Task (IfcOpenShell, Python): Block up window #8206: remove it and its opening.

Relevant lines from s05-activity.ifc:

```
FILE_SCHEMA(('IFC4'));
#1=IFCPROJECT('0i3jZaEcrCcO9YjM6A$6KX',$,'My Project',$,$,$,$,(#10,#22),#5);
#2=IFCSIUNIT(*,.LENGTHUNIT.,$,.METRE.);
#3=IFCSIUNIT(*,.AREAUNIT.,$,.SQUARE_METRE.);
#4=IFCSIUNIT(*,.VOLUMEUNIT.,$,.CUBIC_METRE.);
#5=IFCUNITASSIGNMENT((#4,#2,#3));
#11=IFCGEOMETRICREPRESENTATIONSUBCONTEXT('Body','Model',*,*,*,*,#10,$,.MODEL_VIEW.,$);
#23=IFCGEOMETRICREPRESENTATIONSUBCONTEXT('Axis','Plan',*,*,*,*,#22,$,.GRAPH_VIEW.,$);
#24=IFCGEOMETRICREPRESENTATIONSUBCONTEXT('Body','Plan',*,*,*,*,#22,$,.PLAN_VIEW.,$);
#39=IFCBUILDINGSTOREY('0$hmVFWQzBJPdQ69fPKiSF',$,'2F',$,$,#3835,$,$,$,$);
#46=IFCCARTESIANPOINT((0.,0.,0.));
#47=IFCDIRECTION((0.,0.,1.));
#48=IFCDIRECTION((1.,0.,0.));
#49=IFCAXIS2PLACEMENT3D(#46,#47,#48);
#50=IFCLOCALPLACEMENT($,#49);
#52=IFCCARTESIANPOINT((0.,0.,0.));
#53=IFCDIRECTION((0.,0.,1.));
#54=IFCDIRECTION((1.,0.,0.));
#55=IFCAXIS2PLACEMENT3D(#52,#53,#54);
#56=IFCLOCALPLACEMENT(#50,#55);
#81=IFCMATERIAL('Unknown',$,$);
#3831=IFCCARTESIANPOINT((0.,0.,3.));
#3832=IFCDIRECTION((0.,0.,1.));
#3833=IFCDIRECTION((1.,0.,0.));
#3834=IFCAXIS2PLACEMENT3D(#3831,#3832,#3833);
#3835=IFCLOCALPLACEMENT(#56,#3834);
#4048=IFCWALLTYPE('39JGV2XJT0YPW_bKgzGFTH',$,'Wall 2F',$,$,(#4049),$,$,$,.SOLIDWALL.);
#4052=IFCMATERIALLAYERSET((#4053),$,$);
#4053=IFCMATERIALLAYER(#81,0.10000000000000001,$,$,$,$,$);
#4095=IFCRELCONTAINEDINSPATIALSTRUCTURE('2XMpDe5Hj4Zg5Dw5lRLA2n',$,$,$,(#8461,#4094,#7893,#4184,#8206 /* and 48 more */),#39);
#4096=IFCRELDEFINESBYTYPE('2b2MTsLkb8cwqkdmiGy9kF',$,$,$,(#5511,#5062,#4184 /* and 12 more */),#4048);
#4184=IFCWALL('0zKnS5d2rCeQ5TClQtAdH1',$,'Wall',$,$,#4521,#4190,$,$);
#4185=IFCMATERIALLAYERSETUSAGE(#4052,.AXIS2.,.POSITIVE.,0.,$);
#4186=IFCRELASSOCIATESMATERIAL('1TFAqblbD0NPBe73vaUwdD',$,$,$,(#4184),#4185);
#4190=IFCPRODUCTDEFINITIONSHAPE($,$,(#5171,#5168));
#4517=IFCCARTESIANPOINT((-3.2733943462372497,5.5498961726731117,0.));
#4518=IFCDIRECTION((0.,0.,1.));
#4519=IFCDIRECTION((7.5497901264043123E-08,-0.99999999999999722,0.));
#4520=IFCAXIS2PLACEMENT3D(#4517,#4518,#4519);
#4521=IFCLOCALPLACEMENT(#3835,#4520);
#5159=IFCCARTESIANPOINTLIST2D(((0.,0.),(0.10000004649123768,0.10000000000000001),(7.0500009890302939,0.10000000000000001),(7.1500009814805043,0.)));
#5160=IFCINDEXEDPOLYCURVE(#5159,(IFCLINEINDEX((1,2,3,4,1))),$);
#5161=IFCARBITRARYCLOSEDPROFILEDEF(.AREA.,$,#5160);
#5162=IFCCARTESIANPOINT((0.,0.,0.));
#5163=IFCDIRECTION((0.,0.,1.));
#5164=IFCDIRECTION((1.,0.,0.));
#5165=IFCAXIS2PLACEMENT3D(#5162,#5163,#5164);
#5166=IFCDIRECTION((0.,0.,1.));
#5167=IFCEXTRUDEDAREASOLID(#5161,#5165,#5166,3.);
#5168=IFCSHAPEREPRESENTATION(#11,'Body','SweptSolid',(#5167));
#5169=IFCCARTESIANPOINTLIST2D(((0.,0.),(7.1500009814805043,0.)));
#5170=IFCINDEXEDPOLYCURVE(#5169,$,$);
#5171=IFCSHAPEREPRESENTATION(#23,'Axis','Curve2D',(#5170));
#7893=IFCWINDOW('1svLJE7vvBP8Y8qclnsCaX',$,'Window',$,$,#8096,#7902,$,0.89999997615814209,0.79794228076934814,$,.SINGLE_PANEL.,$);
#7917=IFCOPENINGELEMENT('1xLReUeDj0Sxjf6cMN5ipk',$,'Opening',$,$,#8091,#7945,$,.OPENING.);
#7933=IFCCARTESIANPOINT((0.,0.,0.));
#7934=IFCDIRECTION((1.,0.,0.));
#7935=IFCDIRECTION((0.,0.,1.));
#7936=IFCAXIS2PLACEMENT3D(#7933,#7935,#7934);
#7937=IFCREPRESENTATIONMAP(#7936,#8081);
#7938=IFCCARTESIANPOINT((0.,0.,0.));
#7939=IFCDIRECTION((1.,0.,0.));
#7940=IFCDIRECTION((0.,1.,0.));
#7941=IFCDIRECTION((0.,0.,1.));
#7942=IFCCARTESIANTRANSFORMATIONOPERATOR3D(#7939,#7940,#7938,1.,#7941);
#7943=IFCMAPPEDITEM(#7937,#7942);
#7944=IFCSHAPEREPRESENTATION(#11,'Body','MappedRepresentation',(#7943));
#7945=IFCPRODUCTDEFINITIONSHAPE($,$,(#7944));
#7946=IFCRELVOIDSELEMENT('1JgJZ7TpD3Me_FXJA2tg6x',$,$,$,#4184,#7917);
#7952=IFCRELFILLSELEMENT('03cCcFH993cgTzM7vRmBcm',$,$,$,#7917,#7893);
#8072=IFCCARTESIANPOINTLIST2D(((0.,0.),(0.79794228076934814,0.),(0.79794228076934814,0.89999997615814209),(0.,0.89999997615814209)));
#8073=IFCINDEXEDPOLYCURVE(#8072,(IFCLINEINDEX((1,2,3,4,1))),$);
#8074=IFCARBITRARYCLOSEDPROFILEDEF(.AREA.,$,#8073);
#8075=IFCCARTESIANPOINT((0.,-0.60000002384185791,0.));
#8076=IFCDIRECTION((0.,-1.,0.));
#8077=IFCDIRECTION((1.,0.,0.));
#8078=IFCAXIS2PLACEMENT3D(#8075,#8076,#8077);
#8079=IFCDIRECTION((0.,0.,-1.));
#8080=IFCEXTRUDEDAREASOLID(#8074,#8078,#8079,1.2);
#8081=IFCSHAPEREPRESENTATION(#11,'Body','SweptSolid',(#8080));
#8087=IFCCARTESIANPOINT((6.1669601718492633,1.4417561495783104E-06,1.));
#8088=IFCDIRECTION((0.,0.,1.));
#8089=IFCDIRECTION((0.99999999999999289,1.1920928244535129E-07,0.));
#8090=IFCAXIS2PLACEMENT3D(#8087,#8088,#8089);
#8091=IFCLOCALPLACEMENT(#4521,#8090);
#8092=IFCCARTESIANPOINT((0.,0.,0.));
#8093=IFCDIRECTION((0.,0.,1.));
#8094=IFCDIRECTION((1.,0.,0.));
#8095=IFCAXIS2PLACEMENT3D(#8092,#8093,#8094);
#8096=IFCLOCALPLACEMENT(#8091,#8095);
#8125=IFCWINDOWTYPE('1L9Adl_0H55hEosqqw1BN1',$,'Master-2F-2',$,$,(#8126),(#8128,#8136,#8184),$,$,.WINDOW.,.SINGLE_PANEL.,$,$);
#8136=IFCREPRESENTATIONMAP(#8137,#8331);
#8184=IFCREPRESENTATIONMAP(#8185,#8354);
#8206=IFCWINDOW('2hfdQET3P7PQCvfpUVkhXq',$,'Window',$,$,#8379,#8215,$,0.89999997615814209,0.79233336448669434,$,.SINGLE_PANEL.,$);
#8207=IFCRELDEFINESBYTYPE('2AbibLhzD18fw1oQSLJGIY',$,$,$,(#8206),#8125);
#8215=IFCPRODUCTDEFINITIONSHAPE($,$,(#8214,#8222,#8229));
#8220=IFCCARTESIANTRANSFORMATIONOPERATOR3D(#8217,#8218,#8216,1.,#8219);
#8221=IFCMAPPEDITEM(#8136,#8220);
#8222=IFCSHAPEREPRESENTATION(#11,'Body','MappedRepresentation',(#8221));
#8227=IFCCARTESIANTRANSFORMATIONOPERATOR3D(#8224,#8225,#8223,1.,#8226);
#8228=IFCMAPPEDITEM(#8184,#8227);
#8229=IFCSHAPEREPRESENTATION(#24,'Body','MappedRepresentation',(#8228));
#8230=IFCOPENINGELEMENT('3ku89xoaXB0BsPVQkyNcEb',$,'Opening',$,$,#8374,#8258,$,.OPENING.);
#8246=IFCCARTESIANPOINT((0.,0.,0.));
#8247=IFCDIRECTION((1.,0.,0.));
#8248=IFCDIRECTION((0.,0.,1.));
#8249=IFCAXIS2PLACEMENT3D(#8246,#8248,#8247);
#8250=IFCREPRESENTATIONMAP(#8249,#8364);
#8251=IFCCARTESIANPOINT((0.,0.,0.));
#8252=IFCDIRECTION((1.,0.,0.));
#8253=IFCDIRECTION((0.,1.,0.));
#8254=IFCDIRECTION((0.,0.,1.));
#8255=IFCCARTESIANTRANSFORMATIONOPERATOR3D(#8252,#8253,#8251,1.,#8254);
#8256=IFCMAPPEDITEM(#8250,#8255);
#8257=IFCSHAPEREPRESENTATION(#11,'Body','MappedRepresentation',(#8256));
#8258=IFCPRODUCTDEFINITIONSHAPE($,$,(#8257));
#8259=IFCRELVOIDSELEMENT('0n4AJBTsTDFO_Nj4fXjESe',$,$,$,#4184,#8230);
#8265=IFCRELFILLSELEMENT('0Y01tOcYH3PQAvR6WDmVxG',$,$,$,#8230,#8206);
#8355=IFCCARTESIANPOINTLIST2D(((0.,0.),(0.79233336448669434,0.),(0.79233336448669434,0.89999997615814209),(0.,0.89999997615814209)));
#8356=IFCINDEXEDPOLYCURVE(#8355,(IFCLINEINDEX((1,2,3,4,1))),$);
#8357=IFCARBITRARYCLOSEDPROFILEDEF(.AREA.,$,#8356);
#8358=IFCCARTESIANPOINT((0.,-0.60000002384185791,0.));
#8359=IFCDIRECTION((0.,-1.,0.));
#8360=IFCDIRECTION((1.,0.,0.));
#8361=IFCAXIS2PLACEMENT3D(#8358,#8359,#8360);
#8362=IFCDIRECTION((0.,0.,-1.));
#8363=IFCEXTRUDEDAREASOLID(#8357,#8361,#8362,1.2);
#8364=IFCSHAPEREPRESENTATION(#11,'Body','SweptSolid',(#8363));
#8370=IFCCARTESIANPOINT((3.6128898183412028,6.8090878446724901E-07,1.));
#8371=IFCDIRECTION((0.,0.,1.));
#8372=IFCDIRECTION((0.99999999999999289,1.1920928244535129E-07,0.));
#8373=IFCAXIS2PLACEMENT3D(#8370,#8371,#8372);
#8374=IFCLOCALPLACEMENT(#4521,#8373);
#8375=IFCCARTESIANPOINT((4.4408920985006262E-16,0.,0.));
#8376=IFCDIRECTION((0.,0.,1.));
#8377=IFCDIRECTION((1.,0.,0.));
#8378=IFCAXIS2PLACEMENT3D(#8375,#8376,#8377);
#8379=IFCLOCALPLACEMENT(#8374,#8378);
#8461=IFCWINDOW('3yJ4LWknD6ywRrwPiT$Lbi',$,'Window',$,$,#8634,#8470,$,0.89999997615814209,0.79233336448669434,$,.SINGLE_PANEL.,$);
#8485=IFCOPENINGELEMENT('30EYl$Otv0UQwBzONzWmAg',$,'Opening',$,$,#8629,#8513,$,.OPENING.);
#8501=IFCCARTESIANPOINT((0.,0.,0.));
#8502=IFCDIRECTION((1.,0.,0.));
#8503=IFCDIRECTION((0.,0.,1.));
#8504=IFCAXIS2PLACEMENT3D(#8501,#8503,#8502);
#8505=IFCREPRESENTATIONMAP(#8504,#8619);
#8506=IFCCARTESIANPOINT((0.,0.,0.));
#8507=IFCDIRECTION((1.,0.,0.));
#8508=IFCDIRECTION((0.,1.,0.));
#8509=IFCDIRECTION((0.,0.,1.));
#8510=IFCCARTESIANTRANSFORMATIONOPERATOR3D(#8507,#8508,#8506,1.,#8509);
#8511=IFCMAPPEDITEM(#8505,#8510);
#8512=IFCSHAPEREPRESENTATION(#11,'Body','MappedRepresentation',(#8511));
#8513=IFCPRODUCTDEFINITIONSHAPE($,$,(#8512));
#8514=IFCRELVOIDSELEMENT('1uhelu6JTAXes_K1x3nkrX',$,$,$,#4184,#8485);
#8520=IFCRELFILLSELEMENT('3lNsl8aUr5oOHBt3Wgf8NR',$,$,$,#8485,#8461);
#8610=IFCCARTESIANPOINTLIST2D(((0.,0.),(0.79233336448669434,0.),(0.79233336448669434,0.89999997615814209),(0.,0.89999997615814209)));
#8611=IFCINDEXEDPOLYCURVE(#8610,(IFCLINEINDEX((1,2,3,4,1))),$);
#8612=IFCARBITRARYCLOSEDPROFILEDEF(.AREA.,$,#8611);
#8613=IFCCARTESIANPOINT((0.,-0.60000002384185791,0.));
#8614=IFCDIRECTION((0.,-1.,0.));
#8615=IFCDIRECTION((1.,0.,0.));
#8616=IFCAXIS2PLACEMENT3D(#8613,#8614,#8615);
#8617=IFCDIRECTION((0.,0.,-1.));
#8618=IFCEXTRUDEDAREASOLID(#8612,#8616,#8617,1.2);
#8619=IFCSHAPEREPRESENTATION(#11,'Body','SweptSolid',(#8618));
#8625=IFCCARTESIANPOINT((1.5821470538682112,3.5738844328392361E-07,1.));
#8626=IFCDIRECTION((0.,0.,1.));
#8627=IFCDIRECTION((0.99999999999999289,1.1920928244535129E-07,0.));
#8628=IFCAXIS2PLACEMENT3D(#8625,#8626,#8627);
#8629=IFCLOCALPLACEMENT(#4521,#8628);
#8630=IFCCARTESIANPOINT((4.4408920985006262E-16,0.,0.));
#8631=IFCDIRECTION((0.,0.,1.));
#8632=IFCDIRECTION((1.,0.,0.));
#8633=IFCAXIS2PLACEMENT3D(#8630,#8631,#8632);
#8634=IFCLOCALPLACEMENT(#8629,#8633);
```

```python
import ifcopenshell
import ifcopenshell.api.feature
import ifcopenshell.api.root
import ifcopenshell.geom
import ifcopenshell.util.shape

model = ifcopenshell.open("s05-activity.ifc")
settings = ifcopenshell.geom.settings()


def volume(element):
    """Net volume in cubic metres, openings subtracted."""
    shape = ifcopenshell.geom.create_shape(settings, element)
    return ifcopenshell.util.shape.get_volume(shape.geometry)


window = model.by_guid("2hfdQET3P7PQCvfpUVkhXq")
opening = window.FillsVoids[0].RelatingOpeningElement
wall = opening.VoidsElements[0].RelatingBuildingElement
before = volume(wall)

ifcopenshell.api.root.remove_product(model, product=window)
ifcopenshell.api.feature.remove_feature(model, feature=opening)

after = volume(wall)

print(f"wall volume {before:.3f} -> {after:.3f} m3")

model.write("s05-activity_v2.ifc")
```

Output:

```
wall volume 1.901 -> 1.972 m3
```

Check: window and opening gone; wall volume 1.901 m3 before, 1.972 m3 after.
